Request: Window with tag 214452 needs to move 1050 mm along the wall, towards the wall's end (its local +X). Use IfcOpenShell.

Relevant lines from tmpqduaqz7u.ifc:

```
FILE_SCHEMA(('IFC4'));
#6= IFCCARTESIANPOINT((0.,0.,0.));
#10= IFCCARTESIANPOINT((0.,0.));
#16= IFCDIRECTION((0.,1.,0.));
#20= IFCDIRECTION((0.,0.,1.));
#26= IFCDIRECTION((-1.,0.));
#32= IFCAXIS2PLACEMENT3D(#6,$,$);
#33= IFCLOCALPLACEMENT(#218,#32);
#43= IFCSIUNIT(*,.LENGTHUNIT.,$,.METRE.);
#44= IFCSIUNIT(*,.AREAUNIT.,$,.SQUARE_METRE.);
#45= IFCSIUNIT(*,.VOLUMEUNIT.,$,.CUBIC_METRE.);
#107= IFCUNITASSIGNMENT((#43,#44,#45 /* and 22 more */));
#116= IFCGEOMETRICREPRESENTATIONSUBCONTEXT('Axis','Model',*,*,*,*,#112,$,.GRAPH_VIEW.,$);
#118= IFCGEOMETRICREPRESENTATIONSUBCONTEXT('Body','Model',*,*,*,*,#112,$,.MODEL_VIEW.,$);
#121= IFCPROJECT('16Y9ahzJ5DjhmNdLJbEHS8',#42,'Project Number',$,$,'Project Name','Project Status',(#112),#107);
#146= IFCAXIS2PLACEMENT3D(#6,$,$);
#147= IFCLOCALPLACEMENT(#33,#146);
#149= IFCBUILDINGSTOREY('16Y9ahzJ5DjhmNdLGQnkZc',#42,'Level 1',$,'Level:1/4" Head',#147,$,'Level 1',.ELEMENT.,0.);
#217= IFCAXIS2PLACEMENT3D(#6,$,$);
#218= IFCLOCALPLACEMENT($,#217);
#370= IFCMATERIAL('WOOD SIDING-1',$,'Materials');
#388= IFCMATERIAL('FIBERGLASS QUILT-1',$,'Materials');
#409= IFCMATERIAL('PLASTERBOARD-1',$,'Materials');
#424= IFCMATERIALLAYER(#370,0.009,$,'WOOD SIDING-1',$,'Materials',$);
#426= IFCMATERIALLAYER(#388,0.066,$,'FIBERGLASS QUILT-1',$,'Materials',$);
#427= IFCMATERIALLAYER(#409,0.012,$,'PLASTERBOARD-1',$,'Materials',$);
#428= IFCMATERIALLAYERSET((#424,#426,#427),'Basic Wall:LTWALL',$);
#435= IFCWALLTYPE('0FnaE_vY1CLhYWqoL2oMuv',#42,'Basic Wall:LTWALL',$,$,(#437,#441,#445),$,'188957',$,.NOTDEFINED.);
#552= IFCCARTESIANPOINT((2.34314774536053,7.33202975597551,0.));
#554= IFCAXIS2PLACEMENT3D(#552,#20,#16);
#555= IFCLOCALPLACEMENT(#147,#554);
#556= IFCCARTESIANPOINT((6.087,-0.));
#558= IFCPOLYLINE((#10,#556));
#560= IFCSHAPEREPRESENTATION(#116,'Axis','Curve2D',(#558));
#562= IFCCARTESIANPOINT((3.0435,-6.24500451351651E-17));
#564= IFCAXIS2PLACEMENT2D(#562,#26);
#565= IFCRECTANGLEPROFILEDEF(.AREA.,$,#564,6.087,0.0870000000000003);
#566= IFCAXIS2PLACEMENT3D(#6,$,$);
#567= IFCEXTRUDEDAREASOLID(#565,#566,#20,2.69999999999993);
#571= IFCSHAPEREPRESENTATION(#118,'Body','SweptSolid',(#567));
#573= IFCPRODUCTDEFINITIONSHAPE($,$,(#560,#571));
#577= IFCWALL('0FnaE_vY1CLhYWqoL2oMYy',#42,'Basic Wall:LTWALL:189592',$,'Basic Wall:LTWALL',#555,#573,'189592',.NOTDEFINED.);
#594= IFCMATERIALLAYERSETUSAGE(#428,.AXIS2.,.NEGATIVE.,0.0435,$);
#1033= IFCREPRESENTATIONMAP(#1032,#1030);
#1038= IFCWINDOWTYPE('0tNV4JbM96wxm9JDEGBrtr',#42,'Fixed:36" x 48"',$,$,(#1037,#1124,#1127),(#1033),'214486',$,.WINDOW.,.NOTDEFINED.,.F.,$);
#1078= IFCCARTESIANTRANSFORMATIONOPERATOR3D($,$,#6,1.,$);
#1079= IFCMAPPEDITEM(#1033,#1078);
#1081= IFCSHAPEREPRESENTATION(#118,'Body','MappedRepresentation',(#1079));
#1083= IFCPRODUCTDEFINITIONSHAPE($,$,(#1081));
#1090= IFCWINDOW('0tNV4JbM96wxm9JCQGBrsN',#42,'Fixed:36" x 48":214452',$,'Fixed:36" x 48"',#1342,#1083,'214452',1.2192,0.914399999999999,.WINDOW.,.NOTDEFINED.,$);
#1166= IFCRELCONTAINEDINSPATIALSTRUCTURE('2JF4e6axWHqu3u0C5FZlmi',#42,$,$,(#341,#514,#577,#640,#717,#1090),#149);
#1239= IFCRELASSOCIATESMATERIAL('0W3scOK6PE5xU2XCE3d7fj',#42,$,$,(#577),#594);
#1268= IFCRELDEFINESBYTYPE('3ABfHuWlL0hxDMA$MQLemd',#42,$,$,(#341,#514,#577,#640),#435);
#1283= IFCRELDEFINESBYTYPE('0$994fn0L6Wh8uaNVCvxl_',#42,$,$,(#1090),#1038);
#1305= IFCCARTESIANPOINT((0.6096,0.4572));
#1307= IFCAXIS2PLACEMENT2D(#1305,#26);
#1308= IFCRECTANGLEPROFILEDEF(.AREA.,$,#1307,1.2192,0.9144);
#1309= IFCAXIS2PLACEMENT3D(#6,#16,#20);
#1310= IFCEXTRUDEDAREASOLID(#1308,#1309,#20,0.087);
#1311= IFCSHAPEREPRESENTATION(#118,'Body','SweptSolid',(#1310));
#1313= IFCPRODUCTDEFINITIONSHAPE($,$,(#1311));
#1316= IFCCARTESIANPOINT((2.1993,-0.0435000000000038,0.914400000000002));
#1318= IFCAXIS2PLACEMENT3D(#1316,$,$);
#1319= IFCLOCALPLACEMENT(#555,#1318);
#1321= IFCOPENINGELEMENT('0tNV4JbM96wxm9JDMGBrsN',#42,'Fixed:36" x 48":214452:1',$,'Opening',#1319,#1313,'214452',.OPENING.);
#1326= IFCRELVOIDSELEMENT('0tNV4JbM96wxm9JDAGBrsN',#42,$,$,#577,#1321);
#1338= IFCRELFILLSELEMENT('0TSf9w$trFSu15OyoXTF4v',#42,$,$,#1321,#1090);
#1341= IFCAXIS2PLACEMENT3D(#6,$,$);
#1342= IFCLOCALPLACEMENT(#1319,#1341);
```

```python
import ifcopenshell
import ifcopenshell.api.geometry
import ifcopenshell.util.placement
import ifcopenshell.util.unit

model = ifcopenshell.open("tmpqduaqz7u.ifc")
unit_scale = ifcopenshell.util.unit.calculate_unit_scale(model)

window = model.by_id(1090)
opening = window.FillsVoids[0].RelatingOpeningElement
wall = opening.VoidsElements[0].RelatingBuildingElement

wall_matrix = ifcopenshell.util.placement.get_local_placement(wall.ObjectPlacement)
shift = wall_matrix[:3, 0] * 1.05 / unit_scale
before = ifcopenshell.util.placement.get_local_placement(window.ObjectPlacement)[:3, 3].copy()

# The window is placed relative to its opening, so it follows when the opening moves.
matrix = ifcopenshell.util.placement.get_local_placement(opening.ObjectPlacement)
matrix[:3, 3] += shift
ifcopenshell.api.geometry.edit_object_placement(
    model, product=opening, matrix=matrix, is_si=False, should_transform_children=True
)

after = ifcopenshell.util.placement.get_local_placement(window.ObjectPlacement)[:3, 3]
print("window moved by", (after - before).round(3) + 0.0)

model.write("tmpqduaqz7u_v2.ifc")
```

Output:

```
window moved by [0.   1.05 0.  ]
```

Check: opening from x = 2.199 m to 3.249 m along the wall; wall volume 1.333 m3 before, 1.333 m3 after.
